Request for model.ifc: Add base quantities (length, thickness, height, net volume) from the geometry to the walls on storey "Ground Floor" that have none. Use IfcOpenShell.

First a look at what the model holds.

```python
import ifcopenshell
import ifcopenshell.util.element
import ifcopenshell.util.unit

model = ifcopenshell.open("model.ifc")
print(model.schema)
for unit_type in ("LENGTHUNIT", "AREAUNIT", "VOLUMEUNIT"):
    print(unit_type, ifcopenshell.util.unit.calculate_unit_scale(model, unit_type))
storey = next(s for s in model.by_type("IfcBuildingStorey") if s.Name == "Ground Floor")
walls = [e for e in ifcopenshell.util.element.get_decomposition(storey) if e.is_a("IfcWall")]
for e in sorted(walls, key=lambda e: e.id()):
    print(e.id(), e.is_a(), e.Name, list(ifcopenshell.util.element.get_psets(e, qtos_only=True)), sep=" | ")
```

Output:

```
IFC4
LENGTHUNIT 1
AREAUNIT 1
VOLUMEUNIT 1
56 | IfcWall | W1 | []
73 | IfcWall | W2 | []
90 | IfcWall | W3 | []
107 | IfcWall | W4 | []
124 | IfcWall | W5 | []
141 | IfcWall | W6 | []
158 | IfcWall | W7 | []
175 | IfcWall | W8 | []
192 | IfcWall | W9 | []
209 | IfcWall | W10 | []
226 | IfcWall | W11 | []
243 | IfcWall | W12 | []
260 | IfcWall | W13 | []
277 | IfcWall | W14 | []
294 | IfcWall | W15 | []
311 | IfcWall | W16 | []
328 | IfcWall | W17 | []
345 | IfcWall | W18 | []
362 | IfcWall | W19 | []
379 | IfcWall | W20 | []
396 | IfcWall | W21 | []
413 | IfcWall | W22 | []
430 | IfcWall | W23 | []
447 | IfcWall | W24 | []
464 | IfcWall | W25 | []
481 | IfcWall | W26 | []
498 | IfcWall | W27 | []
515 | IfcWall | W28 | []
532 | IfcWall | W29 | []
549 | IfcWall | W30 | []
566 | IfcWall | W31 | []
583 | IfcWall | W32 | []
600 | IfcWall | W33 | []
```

```python
import ifcopenshell
import ifcopenshell.api.pset
import ifcopenshell.geom
import ifcopenshell.util.element
import ifcopenshell.util.shape
import ifcopenshell.util.unit

model = ifcopenshell.open("model.ifc")
unit_scale = ifcopenshell.util.unit.calculate_unit_scale(model)
volume_scale = ifcopenshell.util.unit.calculate_unit_scale(model, "VOLUMEUNIT")
settings = ifcopenshell.geom.settings()

storey = next(s for s in model.by_type("IfcBuildingStorey") if s.Name == "Ground Floor")
walls = [e for e in ifcopenshell.util.element.get_decomposition(storey) if e.is_a("IfcWall")]

for e in sorted(walls, key=lambda e: e.id()):
    if ifcopenshell.util.element.get_psets(e, qtos_only=True, should_inherit=False):
        continue
    # Geometry comes back in metres, in the element's own axes.
    shape = ifcopenshell.geom.create_shape(settings, e)
    values = {
        "Length": ifcopenshell.util.shape.get_x(shape.geometry) / unit_scale,
        "Width": ifcopenshell.util.shape.get_y(shape.geometry) / unit_scale,
        "Height": ifcopenshell.util.shape.get_z(shape.geometry) / unit_scale,
        "NetVolume": ifcopenshell.util.shape.get_volume(shape.geometry) / volume_scale,
    }
    qto = ifcopenshell.api.pset.add_qto(model, product=e, name="Qto_WallBaseQuantities")
    ifcopenshell.api.pset.edit_qto(model, qto=qto, properties=values)
    print(e.id(), {k: round(v, 3) for k, v in values.items()})

model.write("model_edited.ifc")
```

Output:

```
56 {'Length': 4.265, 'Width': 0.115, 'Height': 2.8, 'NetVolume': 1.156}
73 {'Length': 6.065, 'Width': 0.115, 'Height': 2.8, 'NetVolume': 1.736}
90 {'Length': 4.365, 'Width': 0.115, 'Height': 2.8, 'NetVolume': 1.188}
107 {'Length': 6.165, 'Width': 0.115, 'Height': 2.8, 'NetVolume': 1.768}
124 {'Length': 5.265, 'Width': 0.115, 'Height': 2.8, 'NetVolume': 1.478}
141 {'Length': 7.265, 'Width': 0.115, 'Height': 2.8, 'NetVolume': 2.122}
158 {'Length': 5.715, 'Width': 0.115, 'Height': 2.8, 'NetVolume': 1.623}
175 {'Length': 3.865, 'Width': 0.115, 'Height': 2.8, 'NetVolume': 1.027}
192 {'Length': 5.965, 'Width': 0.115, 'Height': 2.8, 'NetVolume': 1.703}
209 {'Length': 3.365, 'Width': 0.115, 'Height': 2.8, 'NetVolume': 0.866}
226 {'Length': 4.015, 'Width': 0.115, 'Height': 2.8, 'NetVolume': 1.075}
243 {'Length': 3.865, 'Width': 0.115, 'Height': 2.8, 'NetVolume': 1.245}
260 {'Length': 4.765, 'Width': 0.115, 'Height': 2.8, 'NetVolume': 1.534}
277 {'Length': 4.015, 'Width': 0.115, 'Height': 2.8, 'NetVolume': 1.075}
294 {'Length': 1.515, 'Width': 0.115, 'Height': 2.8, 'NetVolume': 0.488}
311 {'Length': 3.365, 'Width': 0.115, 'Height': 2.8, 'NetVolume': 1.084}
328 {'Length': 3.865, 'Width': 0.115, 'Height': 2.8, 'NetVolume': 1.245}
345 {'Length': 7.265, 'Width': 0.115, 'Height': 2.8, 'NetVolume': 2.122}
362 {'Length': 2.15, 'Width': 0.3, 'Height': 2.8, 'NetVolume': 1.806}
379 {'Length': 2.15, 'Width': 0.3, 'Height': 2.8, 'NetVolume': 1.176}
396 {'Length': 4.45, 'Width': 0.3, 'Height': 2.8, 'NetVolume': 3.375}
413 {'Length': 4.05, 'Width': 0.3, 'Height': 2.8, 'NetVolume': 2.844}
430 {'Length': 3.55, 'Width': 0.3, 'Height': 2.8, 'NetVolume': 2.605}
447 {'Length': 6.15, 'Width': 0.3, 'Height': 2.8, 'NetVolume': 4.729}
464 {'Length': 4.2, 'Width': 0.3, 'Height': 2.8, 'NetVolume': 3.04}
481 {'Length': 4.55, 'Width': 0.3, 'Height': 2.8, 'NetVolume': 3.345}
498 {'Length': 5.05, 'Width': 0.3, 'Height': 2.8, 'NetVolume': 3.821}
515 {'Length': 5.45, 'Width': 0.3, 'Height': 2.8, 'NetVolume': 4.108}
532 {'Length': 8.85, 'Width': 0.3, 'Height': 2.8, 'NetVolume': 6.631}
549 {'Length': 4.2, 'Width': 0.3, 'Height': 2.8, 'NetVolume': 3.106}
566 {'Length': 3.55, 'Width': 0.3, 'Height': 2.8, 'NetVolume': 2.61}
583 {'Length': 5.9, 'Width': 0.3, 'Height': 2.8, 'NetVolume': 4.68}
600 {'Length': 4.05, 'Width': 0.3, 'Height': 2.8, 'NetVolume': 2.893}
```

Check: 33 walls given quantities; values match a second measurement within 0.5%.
